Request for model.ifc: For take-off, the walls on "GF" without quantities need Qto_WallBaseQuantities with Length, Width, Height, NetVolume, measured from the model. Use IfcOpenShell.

First a look at what the model holds.

```python
import ifcopenshell
import ifcopenshell.util.element
import ifcopenshell.util.unit

model = ifcopenshell.open("model.ifc")
print(model.schema)
for unit_type in ("LENGTHUNIT", "AREAUNIT", "VOLUMEUNIT"):
    print(unit_type, ifcopenshell.util.unit.calculate_unit_scale(model, unit_type))
storey = next(s for s in model.by_type("IfcBuildingStorey") if s.Name == "GF")
walls = [e for e in ifcopenshell.util.element.get_decomposition(storey) if e.is_a("IfcWall")]
for e in sorted(walls, key=lambda e: e.id()):
    print(e.id(), e.is_a(), e.Name, list(ifcopenshell.util.element.get_psets(e, qtos_only=True)), sep=" | ")
```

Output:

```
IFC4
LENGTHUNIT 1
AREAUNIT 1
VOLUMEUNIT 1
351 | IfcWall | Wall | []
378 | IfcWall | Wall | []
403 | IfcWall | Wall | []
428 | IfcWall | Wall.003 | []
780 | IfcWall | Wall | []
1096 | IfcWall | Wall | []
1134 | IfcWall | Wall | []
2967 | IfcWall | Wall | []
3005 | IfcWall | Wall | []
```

```python
import ifcopenshell
import ifcopenshell.api.pset
import ifcopenshell.geom
import ifcopenshell.util.element
import ifcopenshell.util.shape
import ifcopenshell.util.unit

model = ifcopenshell.open("model.ifc")
unit_scale = ifcopenshell.util.unit.calculate_unit_scale(model)
volume_scale = ifcopenshell.util.unit.calculate_unit_scale(model, "VOLUMEUNIT")
settings = ifcopenshell.geom.settings()

storey = next(s for s in model.by_type("IfcBuildingStorey") if s.Name == "GF")
walls = [e for e in ifcopenshell.util.element.get_decomposition(storey) if e.is_a("IfcWall")]

for e in sorted(walls, key=lambda e: e.id()):
    if ifcopenshell.util.element.get_psets(e, qtos_only=True, should_inherit=False):
        continue
    # Geometry comes back in metres, in the element's own axes.
    shape = ifcopenshell.geom.create_shape(settings, e)
    values = {
        "Length": ifcopenshell.util.shape.get_x(shape.geometry) / unit_scale,
        "Width": ifcopenshell.util.shape.get_y(shape.geometry) / unit_scale,
        "Height": ifcopenshell.util.shape.get_z(shape.geometry) / unit_scale,
        "NetVolume": ifcopenshell.util.shape.get_volume(shape.geometry) / volume_scale,
    }
    qto = ifcopenshell.api.pset.add_qto(model, product=e, name="Qto_WallBaseQuantities")
    ifcopenshell.api.pset.edit_qto(model, qto=qto, properties=values)
    print(e.id(), {k: round(v, 3) for k, v in values.items()})

model.write("model_edited.ifc")
```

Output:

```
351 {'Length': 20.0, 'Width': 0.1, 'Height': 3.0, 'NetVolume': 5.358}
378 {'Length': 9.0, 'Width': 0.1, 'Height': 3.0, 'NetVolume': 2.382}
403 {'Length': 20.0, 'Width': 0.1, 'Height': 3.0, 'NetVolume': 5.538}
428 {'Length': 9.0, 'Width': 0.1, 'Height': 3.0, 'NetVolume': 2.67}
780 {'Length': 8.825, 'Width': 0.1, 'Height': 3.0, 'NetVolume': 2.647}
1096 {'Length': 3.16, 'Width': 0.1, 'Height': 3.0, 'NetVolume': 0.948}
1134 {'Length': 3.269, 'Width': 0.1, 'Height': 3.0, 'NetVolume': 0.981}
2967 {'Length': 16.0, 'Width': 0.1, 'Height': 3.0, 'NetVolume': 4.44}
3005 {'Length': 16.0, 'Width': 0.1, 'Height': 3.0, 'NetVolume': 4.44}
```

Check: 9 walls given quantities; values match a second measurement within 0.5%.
